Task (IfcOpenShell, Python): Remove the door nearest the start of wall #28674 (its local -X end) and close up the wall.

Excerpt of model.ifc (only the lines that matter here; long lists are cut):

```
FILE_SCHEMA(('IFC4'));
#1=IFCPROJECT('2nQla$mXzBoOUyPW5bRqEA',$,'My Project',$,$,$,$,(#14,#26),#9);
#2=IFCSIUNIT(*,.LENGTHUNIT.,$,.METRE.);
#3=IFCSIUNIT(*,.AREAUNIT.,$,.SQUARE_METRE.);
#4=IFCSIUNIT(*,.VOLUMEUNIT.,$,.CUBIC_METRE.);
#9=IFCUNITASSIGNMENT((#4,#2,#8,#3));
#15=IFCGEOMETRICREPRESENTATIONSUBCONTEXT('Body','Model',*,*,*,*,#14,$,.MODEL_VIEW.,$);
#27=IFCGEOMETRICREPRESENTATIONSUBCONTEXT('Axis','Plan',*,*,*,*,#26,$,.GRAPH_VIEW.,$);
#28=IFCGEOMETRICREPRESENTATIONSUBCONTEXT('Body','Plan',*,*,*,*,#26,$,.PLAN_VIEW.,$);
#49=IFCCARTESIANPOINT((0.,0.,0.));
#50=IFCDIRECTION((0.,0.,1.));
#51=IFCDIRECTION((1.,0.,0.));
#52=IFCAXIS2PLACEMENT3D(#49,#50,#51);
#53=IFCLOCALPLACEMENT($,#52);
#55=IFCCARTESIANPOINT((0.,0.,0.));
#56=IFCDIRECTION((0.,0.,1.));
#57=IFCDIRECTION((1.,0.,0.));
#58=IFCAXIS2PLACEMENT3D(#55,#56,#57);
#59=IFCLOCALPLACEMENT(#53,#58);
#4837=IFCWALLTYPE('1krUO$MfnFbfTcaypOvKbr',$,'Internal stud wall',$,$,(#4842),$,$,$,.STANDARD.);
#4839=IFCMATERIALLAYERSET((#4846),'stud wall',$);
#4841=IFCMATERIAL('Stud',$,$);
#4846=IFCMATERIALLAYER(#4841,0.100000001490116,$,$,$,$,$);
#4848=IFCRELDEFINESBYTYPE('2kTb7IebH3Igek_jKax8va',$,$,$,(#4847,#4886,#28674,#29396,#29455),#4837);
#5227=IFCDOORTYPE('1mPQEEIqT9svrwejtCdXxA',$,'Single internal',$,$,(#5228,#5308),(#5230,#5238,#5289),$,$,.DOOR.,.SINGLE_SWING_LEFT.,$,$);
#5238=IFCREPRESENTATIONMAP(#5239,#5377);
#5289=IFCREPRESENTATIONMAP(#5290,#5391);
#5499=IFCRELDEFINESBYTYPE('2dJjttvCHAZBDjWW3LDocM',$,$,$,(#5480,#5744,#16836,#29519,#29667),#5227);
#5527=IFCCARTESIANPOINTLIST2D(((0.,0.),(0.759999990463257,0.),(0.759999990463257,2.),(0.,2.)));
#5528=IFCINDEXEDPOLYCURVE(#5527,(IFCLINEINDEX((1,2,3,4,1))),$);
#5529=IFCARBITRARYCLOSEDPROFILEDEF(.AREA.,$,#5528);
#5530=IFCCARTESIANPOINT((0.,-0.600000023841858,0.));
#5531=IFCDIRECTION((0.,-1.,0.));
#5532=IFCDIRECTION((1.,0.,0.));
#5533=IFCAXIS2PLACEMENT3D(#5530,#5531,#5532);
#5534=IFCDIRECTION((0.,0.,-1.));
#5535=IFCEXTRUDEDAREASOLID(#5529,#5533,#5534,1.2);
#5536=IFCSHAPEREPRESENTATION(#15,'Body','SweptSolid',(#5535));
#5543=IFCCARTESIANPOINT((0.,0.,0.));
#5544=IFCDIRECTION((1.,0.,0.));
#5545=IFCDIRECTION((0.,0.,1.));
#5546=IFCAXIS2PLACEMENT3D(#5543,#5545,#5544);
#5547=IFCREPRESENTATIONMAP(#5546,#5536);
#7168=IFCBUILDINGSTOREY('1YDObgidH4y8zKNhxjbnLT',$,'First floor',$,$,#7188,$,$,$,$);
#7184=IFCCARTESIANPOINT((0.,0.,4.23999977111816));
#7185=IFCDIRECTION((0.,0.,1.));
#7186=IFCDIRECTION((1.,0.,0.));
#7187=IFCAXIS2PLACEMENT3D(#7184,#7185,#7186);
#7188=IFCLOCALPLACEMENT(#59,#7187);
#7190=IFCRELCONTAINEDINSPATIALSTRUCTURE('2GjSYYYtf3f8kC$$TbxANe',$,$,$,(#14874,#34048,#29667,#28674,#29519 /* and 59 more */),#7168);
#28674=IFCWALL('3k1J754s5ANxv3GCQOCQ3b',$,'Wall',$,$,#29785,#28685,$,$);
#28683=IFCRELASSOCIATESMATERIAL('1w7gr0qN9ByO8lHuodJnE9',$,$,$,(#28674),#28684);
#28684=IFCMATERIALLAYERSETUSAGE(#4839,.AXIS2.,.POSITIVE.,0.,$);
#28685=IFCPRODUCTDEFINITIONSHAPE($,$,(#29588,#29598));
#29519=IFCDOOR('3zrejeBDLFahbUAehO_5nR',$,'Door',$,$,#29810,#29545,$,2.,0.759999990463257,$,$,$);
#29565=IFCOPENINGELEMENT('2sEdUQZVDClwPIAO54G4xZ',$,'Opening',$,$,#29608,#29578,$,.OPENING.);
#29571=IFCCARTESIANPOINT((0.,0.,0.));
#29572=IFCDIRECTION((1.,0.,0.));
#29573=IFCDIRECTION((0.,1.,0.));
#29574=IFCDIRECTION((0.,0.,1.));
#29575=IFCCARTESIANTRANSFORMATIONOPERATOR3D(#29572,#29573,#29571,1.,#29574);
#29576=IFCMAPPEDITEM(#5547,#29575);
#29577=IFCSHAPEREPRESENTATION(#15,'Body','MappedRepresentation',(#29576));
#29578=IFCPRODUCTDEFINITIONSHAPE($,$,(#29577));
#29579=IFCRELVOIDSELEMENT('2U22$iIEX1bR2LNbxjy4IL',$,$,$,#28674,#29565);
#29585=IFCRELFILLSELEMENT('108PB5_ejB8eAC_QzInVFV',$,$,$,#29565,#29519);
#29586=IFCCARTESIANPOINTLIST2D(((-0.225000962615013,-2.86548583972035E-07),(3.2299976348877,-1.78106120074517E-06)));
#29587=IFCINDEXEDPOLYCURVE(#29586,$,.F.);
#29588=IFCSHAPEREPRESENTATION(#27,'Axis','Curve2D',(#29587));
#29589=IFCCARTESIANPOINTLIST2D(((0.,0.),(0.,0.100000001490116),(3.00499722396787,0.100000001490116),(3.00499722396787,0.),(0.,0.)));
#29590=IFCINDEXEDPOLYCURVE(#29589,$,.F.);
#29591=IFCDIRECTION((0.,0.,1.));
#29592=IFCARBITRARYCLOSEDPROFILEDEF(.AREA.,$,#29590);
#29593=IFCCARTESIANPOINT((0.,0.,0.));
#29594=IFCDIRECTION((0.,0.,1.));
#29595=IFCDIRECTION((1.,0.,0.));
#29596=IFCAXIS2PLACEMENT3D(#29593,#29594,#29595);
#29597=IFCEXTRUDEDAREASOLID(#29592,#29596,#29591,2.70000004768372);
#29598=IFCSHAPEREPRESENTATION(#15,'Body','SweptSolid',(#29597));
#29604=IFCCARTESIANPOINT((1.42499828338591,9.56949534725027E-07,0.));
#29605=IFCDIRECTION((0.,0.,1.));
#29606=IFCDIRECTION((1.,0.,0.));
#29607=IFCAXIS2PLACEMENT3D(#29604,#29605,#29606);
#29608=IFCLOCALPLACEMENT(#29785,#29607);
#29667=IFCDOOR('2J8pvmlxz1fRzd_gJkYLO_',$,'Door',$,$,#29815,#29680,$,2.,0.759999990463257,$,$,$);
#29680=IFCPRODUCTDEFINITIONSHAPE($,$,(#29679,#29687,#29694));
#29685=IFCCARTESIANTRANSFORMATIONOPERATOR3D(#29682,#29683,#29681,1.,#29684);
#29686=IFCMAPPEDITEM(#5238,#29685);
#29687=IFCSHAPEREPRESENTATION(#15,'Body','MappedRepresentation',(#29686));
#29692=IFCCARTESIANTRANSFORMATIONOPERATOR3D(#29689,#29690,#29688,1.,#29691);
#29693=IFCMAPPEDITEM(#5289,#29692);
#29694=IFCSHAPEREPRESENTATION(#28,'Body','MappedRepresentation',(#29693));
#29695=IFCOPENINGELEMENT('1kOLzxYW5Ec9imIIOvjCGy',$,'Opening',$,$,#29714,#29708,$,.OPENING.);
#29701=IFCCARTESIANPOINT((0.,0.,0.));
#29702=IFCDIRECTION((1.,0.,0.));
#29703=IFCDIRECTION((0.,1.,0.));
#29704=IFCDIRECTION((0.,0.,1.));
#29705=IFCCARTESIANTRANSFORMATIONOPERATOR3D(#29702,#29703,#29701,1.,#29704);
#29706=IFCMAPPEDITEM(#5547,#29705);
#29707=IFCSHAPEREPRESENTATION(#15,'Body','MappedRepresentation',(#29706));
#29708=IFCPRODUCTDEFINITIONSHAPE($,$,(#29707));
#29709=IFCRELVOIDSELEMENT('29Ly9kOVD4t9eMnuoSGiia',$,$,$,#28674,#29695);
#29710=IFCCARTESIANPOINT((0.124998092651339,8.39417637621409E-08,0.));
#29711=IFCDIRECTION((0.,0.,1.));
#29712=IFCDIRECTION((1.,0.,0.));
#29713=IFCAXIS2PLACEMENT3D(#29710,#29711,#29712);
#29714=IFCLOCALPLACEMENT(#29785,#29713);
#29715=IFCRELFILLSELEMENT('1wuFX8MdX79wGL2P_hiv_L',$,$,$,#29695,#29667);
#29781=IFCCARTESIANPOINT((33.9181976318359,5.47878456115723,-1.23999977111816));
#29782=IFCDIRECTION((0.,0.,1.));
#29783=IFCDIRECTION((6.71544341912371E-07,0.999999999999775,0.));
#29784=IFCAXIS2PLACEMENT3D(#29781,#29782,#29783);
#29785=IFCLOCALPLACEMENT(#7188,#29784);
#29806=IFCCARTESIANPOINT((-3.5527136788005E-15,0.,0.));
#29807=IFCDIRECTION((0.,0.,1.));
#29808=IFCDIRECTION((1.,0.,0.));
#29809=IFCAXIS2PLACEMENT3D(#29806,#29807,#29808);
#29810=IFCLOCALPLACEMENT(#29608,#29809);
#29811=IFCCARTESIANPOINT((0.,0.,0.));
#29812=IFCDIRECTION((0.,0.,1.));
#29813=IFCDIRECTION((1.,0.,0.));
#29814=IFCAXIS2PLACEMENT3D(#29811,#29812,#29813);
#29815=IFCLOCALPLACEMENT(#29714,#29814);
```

```python
import ifcopenshell
import ifcopenshell.api.feature
import ifcopenshell.api.root
import ifcopenshell.geom
import ifcopenshell.util.shape

model = ifcopenshell.open("model.ifc")
settings = ifcopenshell.geom.settings()


def volume(element):
    """Net volume in cubic metres, openings subtracted."""
    shape = ifcopenshell.geom.create_shape(settings, element)
    return ifcopenshell.util.shape.get_volume(shape.geometry)


door = model.by_guid("2J8pvmlxz1fRzd_gJkYLO_")
opening = door.FillsVoids[0].RelatingOpeningElement
wall = opening.VoidsElements[0].RelatingBuildingElement
before = volume(wall)

ifcopenshell.api.root.remove_product(model, product=door)
ifcopenshell.api.feature.remove_feature(model, feature=opening)

after = volume(wall)

print(f"wall volume {before:.3f} -> {after:.3f} m3")

model.write("model_updated.ifc")
```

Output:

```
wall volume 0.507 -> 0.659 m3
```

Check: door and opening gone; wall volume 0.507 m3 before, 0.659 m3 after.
